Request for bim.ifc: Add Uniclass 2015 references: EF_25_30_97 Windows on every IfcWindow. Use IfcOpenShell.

First a look at what the model holds.

```python
import ifcopenshell

model = ifcopenshell.open("bim.ifc")
print(model.schema)
print("classifications:", [c.Name for c in model.by_type("IfcClassification")])
for ifc_class in ("IfcDoor", "IfcRoof", "IfcStair", "IfcWall", "IfcWindow"):
    print(ifc_class, len(model.by_type(ifc_class)))
```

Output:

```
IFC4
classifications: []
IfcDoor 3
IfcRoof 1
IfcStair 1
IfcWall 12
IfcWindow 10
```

```python
import ifcopenshell
import ifcopenshell.api.classification

model = ifcopenshell.open("bim.ifc")

system = ifcopenshell.api.classification.add_classification(model, classification="Uniclass 2015")

codes = {
    "IfcWindow": ("EF_25_30_97", "Windows"),
}
for ifc_class, (code, name) in codes.items():
    products = model.by_type(ifc_class)
    ifcopenshell.api.classification.add_reference(
        model, products=products, classification=system, identification=code, name=name
    )
    print(code, len(products))

model.write("bim_edited.ifc")
```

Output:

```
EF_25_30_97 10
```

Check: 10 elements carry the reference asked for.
